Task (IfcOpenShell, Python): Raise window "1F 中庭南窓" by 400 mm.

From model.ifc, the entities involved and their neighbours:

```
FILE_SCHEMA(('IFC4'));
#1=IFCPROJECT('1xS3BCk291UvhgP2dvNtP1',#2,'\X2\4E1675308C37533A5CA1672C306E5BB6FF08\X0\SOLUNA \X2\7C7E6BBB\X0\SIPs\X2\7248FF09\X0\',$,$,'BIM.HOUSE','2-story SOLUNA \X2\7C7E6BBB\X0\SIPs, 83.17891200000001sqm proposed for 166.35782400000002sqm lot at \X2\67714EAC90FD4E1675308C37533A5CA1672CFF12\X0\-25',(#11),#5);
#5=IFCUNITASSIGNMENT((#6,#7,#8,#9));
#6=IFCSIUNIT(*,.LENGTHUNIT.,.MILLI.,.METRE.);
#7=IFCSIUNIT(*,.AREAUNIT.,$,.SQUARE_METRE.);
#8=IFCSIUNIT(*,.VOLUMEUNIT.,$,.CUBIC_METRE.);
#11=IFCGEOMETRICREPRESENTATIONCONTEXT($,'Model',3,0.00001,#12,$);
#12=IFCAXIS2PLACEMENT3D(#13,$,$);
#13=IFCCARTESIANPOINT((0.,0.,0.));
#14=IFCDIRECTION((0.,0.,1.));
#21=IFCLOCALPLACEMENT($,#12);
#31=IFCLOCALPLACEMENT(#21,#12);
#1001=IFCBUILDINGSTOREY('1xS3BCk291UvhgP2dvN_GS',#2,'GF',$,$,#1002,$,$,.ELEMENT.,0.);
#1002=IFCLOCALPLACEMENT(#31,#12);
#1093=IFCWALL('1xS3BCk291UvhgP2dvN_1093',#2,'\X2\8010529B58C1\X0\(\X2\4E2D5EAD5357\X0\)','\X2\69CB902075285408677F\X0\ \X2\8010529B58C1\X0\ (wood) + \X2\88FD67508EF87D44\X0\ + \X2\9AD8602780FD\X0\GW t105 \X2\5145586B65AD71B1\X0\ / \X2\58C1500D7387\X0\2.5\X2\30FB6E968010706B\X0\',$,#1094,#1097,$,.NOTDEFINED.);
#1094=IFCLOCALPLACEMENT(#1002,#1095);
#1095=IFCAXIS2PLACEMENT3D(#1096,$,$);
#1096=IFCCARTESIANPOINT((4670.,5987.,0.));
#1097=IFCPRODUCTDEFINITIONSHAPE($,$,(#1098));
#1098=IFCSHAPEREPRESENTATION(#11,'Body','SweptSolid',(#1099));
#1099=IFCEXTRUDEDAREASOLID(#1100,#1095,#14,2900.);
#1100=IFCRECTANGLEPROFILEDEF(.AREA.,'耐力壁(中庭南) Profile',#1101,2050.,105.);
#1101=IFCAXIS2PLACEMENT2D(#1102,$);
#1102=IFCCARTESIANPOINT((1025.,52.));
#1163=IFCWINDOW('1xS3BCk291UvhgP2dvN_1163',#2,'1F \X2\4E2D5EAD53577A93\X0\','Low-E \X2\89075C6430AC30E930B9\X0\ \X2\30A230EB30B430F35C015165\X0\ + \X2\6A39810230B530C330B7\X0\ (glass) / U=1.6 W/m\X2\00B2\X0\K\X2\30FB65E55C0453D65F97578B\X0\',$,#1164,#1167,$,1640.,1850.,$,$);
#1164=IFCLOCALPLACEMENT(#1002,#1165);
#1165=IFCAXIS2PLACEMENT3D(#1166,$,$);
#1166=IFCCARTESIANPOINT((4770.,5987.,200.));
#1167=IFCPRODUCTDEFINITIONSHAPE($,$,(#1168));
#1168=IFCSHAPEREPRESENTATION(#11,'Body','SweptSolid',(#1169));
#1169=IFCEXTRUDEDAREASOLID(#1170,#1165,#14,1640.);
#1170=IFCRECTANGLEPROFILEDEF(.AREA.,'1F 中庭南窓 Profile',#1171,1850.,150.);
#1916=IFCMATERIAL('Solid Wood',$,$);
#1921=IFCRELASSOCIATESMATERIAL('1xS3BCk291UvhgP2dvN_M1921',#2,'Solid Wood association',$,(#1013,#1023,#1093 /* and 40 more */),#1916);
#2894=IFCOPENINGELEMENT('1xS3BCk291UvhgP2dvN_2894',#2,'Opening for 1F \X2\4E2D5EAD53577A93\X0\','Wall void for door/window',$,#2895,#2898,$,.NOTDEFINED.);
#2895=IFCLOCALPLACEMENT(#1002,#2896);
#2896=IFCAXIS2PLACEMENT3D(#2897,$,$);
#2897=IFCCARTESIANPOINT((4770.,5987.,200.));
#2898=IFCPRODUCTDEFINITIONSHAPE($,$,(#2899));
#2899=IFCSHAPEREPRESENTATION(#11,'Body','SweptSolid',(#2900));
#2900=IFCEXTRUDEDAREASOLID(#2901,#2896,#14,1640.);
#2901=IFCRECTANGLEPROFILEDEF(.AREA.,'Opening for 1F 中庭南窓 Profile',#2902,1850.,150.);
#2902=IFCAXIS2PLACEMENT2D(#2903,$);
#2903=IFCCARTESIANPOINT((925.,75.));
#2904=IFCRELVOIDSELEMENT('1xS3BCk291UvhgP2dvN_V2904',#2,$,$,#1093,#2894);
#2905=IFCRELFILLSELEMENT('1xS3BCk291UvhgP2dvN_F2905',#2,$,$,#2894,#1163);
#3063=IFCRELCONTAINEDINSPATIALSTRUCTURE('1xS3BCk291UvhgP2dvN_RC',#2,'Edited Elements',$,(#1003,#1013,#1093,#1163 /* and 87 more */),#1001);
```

```python
import numpy as np
import ifcopenshell
import ifcopenshell.api.geometry
import ifcopenshell.util.placement
import ifcopenshell.util.unit

model = ifcopenshell.open("model.ifc")
unit_scale = ifcopenshell.util.unit.calculate_unit_scale(model)

window = model.by_id(1163)
opening = window.FillsVoids[0].RelatingOpeningElement
dz = 400.0

shift = np.array([0.0, 0.0, dz])
# The window is not placed relative to its opening, so move both.
for product in (opening, window):
    matrix = ifcopenshell.util.placement.get_local_placement(product.ObjectPlacement)
    matrix[:3, 3] += shift
    ifcopenshell.api.geometry.edit_object_placement(model, product=product, matrix=matrix, is_si=False)

print(f"moved by {dz * unit_scale:+.3f} m")

model.write("model-out.ifc")
```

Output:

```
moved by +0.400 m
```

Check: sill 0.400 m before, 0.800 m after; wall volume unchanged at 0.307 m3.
